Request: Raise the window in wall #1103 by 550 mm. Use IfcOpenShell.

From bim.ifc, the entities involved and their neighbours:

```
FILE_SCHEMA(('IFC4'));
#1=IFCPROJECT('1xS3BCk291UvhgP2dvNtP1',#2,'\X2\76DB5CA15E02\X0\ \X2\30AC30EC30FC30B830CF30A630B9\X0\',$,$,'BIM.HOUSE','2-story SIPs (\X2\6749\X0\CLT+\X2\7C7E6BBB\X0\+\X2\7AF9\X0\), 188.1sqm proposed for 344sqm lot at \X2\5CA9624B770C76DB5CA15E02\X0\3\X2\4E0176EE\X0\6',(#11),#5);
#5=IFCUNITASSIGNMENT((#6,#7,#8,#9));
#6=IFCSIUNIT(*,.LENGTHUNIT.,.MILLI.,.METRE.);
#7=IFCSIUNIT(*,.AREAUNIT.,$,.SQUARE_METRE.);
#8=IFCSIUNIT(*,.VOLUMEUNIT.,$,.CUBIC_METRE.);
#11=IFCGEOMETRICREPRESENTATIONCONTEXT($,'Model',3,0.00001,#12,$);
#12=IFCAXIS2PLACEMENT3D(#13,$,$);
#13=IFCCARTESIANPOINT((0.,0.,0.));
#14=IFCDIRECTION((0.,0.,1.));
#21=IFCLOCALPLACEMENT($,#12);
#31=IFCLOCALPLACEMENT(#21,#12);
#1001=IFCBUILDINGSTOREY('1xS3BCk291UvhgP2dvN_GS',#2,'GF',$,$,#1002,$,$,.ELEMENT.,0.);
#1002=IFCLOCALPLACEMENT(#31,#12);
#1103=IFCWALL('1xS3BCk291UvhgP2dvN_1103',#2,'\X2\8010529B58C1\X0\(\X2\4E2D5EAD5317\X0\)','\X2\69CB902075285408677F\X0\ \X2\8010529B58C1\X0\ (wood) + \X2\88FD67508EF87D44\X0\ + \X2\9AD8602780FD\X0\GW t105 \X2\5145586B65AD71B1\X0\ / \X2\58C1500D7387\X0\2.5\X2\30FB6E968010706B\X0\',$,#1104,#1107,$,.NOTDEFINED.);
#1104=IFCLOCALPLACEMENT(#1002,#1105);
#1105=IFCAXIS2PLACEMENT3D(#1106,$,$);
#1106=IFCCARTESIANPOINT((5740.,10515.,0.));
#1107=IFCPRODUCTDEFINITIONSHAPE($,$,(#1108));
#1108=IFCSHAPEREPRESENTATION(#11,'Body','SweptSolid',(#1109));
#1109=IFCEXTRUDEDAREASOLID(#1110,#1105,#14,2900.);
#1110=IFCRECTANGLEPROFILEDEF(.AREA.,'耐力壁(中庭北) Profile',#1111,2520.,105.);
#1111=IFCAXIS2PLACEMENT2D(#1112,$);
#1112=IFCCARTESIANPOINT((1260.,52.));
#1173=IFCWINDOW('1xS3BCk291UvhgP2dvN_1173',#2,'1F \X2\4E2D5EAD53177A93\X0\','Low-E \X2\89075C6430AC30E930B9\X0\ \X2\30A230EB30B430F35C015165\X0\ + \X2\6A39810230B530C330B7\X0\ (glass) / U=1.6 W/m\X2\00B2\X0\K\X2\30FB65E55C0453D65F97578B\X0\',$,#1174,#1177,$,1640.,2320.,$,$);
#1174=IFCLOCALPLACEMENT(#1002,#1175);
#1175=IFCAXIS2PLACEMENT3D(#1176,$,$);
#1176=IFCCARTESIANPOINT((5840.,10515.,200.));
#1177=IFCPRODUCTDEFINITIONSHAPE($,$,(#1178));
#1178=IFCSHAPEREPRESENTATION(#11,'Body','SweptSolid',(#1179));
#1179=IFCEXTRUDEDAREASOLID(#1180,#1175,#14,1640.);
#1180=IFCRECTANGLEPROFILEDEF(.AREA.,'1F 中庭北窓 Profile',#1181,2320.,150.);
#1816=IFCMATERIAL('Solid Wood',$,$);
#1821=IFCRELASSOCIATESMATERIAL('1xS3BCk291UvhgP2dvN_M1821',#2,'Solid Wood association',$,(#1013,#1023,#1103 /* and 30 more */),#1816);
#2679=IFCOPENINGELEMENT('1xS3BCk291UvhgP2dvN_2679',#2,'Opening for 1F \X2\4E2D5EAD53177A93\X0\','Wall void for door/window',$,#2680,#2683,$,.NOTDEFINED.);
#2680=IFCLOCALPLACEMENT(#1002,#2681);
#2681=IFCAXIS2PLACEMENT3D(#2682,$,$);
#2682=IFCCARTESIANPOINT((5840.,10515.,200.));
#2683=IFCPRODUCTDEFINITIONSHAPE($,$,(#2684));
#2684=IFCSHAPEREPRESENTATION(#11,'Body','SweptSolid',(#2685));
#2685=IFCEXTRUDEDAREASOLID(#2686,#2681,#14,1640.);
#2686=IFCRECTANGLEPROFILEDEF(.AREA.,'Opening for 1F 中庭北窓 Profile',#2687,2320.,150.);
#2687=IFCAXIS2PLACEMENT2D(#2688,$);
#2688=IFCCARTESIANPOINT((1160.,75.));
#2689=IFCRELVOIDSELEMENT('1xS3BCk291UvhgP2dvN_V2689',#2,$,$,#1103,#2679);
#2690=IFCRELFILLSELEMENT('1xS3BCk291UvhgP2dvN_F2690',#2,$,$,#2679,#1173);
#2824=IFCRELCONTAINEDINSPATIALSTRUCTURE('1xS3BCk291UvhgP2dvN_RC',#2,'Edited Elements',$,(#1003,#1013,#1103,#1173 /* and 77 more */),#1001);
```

```python
import numpy as np
import ifcopenshell
import ifcopenshell.api.geometry
import ifcopenshell.util.placement
import ifcopenshell.util.unit

model = ifcopenshell.open("bim.ifc")
unit_scale = ifcopenshell.util.unit.calculate_unit_scale(model)

window = model.by_guid("1xS3BCk291UvhgP2dvN_1173")
opening = window.FillsVoids[0].RelatingOpeningElement
dz = 550.0

shift = np.array([0.0, 0.0, dz])
# The window is not placed relative to its opening, so move both.
for product in (opening, window):
    matrix = ifcopenshell.util.placement.get_local_placement(product.ObjectPlacement)
    matrix[:3, 3] += shift
    ifcopenshell.api.geometry.edit_object_placement(model, product=product, matrix=matrix, is_si=False)

print(f"moved by {dz * unit_scale:+.3f} m")

model.write("bim-out.ifc")
```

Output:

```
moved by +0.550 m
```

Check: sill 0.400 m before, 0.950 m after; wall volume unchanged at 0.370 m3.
